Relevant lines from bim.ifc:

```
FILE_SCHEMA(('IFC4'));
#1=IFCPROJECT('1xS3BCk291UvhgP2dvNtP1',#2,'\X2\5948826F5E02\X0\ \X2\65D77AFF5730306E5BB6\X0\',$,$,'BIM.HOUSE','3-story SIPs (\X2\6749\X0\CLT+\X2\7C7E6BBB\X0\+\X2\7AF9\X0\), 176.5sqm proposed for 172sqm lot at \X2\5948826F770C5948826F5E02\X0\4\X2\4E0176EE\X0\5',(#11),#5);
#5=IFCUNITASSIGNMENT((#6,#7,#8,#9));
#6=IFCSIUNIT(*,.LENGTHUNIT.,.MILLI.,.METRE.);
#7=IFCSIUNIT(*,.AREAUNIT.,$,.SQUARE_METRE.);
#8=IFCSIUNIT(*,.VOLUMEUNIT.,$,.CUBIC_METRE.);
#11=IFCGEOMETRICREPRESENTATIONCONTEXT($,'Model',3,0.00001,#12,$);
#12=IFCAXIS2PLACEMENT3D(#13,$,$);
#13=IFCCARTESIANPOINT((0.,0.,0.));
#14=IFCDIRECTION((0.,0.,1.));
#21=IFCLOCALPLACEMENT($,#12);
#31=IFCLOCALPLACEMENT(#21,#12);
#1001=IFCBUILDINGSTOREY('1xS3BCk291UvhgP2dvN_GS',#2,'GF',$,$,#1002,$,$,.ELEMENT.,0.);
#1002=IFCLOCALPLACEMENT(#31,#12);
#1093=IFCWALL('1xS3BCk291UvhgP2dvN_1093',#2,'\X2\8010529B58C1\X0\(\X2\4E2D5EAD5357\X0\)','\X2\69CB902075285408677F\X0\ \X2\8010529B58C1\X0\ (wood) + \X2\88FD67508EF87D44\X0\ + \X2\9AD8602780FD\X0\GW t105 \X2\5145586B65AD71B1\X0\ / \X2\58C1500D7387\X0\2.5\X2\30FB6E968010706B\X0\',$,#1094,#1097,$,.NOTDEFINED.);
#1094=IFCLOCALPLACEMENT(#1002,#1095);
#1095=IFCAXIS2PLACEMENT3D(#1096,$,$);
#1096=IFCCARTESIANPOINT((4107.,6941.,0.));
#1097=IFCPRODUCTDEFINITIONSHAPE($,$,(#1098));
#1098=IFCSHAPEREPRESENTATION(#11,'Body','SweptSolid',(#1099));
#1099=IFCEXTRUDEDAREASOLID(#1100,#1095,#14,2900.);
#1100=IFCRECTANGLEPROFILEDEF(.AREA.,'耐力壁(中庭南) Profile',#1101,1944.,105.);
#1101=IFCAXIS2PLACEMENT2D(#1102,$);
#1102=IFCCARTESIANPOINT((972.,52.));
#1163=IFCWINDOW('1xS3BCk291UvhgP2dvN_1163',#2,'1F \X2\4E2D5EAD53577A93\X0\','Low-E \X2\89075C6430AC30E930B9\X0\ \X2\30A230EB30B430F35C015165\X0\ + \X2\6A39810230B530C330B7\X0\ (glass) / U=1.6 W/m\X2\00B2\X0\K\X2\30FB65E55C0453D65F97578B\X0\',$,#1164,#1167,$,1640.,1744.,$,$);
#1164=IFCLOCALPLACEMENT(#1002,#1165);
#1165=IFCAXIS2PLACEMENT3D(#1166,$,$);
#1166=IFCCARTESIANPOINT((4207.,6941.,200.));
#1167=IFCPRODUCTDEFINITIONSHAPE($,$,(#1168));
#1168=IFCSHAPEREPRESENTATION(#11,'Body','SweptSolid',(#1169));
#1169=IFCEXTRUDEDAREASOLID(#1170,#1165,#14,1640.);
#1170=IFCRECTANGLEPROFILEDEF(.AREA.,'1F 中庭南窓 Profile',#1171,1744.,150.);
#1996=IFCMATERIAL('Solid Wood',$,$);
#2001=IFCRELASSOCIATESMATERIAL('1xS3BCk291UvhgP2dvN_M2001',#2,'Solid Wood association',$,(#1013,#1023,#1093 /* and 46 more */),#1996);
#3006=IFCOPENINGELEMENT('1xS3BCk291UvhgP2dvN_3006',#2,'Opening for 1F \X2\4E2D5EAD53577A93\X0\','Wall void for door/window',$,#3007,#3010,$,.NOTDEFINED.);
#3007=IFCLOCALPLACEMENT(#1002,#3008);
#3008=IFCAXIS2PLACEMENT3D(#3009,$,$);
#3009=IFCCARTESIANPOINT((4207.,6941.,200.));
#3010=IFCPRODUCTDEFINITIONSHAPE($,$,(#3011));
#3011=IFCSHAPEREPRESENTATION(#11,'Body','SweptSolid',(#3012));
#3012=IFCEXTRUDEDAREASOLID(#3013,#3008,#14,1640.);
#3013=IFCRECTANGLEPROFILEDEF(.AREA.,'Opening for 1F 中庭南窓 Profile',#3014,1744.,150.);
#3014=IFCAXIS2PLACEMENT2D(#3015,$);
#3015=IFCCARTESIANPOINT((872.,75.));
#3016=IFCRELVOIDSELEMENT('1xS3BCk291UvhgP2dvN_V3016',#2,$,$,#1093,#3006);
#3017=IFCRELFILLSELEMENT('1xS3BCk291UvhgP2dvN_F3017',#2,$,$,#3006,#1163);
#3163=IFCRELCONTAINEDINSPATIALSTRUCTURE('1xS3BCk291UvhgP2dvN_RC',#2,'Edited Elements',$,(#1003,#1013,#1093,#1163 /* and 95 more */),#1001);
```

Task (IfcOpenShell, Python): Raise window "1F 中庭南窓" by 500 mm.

```python
import numpy as np
import ifcopenshell
import ifcopenshell.api.geometry
import ifcopenshell.util.placement
import ifcopenshell.util.unit

model = ifcopenshell.open("bim.ifc")
unit_scale = ifcopenshell.util.unit.calculate_unit_scale(model)

window = model.by_guid("1xS3BCk291UvhgP2dvN_1163")
opening = window.FillsVoids[0].RelatingOpeningElement
dz = 0.5 / unit_scale

shift = np.array([0.0, 0.0, dz])
# The window is not placed relative to its opening, so move both.
for product in (opening, window):
    matrix = ifcopenshell.util.placement.get_local_placement(product.ObjectPlacement)
    matrix[:3, 3] += shift
    ifcopenshell.api.geometry.edit_object_placement(model, product=product, matrix=matrix, is_si=False)

print(f"moved by {dz * unit_scale:+.3f} m")

model.write("bim_v2.ifc")
```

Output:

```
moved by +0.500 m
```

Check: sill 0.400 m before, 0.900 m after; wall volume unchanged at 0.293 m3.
